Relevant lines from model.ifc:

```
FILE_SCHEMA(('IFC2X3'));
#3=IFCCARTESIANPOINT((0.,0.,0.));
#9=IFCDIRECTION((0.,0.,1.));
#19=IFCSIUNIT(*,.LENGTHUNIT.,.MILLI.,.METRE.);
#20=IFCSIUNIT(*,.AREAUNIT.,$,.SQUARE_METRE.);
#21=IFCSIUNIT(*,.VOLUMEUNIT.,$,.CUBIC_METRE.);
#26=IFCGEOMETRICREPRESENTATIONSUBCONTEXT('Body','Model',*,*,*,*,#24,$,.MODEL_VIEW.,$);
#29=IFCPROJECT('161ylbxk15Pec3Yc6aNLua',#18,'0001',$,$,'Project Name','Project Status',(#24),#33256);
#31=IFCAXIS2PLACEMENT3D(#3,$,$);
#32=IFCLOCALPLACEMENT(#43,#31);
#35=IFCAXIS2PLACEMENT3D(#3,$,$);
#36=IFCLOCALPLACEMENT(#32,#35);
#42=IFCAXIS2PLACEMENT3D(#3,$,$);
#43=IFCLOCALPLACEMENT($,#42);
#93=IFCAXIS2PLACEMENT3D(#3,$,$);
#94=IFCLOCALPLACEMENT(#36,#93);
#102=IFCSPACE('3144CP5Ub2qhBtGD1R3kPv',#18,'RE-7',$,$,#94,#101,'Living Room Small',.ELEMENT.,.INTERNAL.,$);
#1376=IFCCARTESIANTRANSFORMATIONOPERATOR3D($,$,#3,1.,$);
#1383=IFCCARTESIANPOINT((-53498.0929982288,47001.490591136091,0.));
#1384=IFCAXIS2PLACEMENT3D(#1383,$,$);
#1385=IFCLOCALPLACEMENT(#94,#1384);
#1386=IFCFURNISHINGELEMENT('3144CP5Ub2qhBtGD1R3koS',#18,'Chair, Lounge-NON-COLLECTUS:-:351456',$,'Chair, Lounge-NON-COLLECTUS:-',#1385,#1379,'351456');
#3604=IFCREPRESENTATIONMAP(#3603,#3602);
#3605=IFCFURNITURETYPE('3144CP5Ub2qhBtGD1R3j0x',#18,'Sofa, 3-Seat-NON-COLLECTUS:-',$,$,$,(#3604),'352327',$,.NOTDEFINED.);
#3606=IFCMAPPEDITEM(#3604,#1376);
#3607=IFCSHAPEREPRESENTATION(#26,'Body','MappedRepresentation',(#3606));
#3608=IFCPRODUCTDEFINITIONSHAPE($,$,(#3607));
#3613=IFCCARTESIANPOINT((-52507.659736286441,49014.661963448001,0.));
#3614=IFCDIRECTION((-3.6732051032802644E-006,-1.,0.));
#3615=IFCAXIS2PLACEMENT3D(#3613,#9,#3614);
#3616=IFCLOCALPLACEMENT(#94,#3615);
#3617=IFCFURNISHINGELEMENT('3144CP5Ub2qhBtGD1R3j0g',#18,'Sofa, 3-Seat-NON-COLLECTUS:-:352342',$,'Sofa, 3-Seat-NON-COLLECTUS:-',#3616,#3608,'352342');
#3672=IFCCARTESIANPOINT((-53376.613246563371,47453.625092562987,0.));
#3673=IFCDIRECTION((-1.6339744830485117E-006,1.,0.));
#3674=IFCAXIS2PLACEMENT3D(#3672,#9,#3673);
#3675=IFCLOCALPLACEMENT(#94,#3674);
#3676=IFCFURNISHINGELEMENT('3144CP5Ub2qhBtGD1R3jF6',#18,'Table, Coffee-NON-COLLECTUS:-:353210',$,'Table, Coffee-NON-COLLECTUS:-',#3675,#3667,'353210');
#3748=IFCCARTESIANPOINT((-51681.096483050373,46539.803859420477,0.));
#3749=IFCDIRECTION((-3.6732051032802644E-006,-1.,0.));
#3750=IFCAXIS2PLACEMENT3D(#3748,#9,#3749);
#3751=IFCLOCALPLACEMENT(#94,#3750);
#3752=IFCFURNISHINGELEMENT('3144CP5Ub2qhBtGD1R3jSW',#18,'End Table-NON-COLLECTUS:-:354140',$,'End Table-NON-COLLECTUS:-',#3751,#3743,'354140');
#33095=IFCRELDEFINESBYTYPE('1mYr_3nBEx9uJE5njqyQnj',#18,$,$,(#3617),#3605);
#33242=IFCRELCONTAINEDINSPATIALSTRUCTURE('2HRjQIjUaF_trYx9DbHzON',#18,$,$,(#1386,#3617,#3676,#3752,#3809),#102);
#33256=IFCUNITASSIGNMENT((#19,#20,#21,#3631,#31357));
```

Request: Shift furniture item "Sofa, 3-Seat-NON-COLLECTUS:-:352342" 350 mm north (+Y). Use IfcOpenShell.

```python
import ifcopenshell
import ifcopenshell.api.geometry
import ifcopenshell.util.placement

model = ifcopenshell.open("model.ifc")

item = model.by_guid("3144CP5Ub2qhBtGD1R3j0g")
matrix = ifcopenshell.util.placement.get_local_placement(item.ObjectPlacement)
matrix[1, 3] += 350.0
ifcopenshell.api.geometry.edit_object_placement(model, product=item, matrix=matrix, is_si=False)

print(ifcopenshell.util.placement.get_local_placement(item.ObjectPlacement).round(3) + 0.0)

model.write("model_rev.ifc")
```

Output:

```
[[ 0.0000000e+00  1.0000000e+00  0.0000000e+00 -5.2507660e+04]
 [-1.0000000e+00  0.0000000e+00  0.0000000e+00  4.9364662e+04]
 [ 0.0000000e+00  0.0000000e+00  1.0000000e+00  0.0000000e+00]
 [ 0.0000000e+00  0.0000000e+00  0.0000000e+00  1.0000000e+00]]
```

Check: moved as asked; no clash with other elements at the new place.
